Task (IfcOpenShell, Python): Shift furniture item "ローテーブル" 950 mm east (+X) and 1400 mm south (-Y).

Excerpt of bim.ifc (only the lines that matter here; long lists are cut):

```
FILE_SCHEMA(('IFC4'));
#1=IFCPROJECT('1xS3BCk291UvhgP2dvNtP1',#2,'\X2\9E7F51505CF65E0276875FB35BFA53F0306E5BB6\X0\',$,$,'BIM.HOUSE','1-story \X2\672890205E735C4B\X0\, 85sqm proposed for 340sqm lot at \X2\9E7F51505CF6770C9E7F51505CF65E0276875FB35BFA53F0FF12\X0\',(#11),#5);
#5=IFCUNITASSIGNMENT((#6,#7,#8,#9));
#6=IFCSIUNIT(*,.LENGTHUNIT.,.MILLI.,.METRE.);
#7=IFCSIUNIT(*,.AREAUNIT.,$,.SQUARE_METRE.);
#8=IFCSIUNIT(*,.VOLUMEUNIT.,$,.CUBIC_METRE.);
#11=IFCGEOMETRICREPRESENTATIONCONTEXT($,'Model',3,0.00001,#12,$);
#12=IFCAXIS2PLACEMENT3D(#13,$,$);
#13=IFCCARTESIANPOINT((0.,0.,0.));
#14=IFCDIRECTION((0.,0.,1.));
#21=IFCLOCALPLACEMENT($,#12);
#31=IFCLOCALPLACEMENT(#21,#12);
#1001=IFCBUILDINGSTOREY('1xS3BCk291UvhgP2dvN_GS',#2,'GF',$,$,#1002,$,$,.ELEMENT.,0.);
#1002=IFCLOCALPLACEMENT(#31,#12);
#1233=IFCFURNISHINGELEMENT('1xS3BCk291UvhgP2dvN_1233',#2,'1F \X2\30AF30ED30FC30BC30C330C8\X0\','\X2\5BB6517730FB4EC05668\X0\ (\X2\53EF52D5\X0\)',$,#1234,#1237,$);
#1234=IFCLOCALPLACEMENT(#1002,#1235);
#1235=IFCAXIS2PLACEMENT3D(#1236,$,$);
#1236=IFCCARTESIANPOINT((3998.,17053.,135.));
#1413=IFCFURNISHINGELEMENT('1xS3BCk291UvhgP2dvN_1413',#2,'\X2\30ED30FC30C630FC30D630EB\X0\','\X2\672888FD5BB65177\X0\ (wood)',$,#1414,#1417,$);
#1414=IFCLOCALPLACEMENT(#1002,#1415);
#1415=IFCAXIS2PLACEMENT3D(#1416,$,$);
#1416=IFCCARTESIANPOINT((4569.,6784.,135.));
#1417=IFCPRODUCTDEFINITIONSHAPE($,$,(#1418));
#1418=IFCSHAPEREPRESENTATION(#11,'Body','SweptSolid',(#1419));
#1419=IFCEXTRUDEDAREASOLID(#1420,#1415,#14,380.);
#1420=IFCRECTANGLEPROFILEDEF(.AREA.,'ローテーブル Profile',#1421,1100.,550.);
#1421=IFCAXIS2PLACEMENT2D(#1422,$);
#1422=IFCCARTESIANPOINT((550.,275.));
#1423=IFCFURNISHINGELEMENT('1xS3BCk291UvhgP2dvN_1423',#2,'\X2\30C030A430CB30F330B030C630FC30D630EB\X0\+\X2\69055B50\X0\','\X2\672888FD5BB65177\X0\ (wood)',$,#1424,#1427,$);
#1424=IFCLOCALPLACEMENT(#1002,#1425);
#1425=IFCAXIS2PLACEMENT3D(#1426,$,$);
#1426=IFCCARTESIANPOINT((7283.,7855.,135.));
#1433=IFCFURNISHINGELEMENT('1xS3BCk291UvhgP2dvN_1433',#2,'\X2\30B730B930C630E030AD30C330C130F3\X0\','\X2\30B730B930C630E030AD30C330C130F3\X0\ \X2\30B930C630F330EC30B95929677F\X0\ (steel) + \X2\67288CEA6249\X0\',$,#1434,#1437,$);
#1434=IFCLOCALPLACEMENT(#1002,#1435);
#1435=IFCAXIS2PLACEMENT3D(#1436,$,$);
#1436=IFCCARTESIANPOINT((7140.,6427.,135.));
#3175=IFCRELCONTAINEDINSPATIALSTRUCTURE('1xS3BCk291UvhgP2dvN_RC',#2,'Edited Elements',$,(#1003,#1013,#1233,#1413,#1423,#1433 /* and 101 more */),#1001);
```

```python
import ifcopenshell
import ifcopenshell.api.geometry
import ifcopenshell.util.placement

model = ifcopenshell.open("bim.ifc")

item = model.by_guid("1xS3BCk291UvhgP2dvN_1413")
matrix = ifcopenshell.util.placement.get_local_placement(item.ObjectPlacement)
matrix[0, 3] += 950.0
matrix[1, 3] -= 1400.0
ifcopenshell.api.geometry.edit_object_placement(model, product=item, matrix=matrix, is_si=False)

print(ifcopenshell.util.placement.get_local_placement(item.ObjectPlacement).round(3) + 0.0)

model.write("bim_edited.ifc")
```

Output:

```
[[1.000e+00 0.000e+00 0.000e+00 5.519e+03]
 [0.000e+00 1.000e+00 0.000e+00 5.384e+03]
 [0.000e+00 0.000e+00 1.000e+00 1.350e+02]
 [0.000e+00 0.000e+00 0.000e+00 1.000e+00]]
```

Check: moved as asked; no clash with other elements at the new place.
